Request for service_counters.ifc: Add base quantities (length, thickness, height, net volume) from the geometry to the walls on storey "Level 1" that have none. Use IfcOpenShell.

First a look at what the model holds.

```python
import ifcopenshell
import ifcopenshell.util.element
import ifcopenshell.util.unit

model = ifcopenshell.open("service_counters.ifc")
print(model.schema)
for unit_type in ("LENGTHUNIT", "AREAUNIT", "VOLUMEUNIT"):
    print(unit_type, ifcopenshell.util.unit.calculate_unit_scale(model, unit_type))
storey = next(s for s in model.by_type("IfcBuildingStorey") if s.Name == "Level 1")
walls = [e for e in ifcopenshell.util.element.get_decomposition(storey) if e.is_a("IfcWall")]
for e in sorted(walls, key=lambda e: e.id()):
    print(e.id(), e.is_a(), e.Name, list(ifcopenshell.util.element.get_psets(e, qtos_only=True)), sep=" | ")
```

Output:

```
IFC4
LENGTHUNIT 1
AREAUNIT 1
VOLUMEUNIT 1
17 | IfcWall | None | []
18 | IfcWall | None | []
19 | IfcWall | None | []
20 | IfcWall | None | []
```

```python
import ifcopenshell
import ifcopenshell.api.pset
import ifcopenshell.geom
import ifcopenshell.util.element
import ifcopenshell.util.shape
import ifcopenshell.util.unit

model = ifcopenshell.open("service_counters.ifc")
unit_scale = ifcopenshell.util.unit.calculate_unit_scale(model)
volume_scale = ifcopenshell.util.unit.calculate_unit_scale(model, "VOLUMEUNIT")
settings = ifcopenshell.geom.settings()

storey = next(s for s in model.by_type("IfcBuildingStorey") if s.Name == "Level 1")
walls = [e for e in ifcopenshell.util.element.get_decomposition(storey) if e.is_a("IfcWall")]

for e in sorted(walls, key=lambda e: e.id()):
    if ifcopenshell.util.element.get_psets(e, qtos_only=True, should_inherit=False):
        continue
    # Geometry comes back in metres, in the element's own axes.
    shape = ifcopenshell.geom.create_shape(settings, e)
    values = {
        "Length": ifcopenshell.util.shape.get_x(shape.geometry) / unit_scale,
        "Width": ifcopenshell.util.shape.get_y(shape.geometry) / unit_scale,
        "Height": ifcopenshell.util.shape.get_z(shape.geometry) / unit_scale,
        "NetVolume": ifcopenshell.util.shape.get_volume(shape.geometry) / volume_scale,
    }
    qto = ifcopenshell.api.pset.add_qto(model, product=e, name="Qto_WallBaseQuantities")
    ifcopenshell.api.pset.edit_qto(model, qto=qto, properties=values)
    print(e.id(), {k: round(v, 3) for k, v in values.items()})

model.write("service_counters_rev.ifc")
```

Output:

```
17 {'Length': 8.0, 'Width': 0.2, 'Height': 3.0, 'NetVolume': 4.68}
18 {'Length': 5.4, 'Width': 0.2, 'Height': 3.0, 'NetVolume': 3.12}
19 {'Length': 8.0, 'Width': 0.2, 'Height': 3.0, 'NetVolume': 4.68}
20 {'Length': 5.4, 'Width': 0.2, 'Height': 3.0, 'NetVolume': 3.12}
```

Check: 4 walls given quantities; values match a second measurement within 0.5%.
